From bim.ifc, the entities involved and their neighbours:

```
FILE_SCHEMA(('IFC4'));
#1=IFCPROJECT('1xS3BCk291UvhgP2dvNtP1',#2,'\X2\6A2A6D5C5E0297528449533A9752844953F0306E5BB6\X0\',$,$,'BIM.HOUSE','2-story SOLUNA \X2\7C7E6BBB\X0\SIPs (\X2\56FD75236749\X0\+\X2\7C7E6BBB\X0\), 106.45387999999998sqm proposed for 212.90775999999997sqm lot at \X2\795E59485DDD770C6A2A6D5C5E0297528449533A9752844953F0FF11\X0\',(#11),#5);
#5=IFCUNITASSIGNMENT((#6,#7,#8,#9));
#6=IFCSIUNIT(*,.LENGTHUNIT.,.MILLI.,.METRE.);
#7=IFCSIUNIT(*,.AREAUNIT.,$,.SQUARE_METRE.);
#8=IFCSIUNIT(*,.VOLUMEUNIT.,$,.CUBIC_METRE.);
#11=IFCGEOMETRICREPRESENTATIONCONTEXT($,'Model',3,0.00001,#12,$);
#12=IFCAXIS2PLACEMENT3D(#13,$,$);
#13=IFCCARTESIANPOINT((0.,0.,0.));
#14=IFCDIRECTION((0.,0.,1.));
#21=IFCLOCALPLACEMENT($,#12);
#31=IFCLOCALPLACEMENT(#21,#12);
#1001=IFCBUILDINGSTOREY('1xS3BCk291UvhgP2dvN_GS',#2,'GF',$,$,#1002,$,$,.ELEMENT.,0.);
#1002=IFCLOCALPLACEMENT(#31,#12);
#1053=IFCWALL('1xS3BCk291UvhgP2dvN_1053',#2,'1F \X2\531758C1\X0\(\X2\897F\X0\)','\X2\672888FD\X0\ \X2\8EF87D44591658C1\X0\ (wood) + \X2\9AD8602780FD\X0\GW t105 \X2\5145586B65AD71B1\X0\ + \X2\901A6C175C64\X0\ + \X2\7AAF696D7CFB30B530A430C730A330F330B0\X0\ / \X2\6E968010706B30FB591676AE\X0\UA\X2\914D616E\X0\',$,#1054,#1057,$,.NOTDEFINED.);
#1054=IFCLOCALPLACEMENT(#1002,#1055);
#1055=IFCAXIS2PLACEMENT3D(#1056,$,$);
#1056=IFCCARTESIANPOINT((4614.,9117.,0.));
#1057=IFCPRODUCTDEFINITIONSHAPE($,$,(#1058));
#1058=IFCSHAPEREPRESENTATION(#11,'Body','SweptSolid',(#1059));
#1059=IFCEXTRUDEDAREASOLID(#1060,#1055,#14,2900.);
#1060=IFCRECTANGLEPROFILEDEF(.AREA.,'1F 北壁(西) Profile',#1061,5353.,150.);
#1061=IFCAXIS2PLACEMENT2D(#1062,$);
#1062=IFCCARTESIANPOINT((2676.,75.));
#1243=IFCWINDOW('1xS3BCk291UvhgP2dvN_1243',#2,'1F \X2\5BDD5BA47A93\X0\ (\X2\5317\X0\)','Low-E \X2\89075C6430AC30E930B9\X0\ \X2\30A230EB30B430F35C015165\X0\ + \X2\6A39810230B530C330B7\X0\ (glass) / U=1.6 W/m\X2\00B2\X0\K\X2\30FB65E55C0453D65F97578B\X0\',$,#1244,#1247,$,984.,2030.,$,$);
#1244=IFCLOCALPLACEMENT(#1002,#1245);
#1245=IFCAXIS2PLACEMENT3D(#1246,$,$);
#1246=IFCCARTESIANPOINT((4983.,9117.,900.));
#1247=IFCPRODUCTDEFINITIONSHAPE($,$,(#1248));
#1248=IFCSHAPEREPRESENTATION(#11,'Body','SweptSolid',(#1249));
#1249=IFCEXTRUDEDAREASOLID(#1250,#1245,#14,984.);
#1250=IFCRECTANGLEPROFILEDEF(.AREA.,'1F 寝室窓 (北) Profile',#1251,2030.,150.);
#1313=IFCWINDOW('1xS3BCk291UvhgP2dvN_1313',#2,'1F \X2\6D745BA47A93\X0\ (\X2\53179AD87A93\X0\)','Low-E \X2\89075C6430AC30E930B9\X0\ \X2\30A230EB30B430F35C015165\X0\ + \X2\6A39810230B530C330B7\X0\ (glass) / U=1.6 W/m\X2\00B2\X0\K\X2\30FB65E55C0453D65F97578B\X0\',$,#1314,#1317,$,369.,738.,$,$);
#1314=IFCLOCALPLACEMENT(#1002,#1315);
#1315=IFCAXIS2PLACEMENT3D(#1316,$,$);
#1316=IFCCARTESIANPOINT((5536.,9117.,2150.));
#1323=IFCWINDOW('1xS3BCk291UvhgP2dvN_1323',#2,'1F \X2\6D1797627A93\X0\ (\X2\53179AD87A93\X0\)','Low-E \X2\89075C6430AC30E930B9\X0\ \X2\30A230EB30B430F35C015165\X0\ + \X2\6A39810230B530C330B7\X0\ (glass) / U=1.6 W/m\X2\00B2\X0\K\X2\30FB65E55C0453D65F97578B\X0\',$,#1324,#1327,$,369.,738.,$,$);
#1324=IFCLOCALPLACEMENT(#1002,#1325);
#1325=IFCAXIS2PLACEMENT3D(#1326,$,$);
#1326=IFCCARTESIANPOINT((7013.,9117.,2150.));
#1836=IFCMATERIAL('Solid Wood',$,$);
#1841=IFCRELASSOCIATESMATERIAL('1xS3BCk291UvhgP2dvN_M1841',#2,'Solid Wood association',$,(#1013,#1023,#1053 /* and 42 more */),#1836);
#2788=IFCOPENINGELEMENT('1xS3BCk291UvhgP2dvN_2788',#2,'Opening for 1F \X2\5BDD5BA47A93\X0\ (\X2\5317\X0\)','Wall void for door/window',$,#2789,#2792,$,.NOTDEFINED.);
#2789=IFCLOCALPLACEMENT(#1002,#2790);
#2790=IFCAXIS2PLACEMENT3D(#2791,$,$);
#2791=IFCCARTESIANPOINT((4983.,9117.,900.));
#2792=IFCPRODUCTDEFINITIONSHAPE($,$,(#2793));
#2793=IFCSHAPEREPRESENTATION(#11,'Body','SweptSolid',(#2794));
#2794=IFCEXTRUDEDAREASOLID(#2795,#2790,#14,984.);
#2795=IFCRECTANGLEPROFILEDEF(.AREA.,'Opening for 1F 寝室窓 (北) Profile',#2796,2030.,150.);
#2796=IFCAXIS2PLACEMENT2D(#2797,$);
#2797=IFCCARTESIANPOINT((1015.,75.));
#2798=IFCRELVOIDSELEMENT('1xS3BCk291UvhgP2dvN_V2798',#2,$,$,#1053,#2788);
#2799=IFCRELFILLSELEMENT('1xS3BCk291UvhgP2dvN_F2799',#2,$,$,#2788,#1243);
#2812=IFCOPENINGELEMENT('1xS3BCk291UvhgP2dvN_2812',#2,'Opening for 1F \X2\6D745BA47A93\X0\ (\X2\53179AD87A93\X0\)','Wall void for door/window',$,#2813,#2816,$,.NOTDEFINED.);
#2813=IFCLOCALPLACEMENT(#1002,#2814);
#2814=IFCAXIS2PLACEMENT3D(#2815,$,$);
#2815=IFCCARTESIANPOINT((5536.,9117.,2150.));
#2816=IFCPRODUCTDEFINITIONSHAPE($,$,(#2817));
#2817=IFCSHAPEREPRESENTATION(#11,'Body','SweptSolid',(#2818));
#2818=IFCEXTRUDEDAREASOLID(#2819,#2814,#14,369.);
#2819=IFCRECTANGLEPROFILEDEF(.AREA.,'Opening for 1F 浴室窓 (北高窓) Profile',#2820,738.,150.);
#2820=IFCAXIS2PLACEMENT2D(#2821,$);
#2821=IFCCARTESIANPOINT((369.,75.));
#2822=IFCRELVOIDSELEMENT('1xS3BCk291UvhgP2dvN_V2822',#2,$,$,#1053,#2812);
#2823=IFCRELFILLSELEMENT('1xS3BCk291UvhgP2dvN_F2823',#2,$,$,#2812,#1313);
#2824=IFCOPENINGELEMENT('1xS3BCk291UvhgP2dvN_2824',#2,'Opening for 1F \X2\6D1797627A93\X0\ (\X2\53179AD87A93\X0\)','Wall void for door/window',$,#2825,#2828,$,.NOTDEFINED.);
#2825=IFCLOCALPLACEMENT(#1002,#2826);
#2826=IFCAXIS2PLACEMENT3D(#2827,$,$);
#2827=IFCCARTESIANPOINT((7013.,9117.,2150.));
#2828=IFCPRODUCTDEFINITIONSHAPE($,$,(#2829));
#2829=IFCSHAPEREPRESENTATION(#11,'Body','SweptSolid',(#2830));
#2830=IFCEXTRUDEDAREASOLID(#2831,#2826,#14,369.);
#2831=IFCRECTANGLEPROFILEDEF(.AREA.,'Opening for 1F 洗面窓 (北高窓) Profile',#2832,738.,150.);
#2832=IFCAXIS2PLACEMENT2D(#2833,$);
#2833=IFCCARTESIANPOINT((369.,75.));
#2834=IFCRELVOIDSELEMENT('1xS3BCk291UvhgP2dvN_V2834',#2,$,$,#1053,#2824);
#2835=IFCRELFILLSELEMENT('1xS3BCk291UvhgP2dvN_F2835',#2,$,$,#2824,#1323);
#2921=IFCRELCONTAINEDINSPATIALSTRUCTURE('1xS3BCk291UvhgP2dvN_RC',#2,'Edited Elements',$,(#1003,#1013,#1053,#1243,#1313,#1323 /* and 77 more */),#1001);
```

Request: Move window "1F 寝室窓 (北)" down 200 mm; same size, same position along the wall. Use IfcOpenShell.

```python
import numpy as np
import ifcopenshell
import ifcopenshell.api.geometry
import ifcopenshell.util.placement
import ifcopenshell.util.unit

model = ifcopenshell.open("bim.ifc")
unit_scale = ifcopenshell.util.unit.calculate_unit_scale(model)

window = model.by_guid("1xS3BCk291UvhgP2dvN_1243")
opening = window.FillsVoids[0].RelatingOpeningElement
dz = -0.2 / unit_scale

shift = np.array([0.0, 0.0, dz])
# The window is not placed relative to its opening, so move both.
for product in (opening, window):
    matrix = ifcopenshell.util.placement.get_local_placement(product.ObjectPlacement)
    matrix[:3, 3] += shift
    ifcopenshell.api.geometry.edit_object_placement(model, product=product, matrix=matrix, is_si=False)

print(f"moved by {dz * unit_scale:+.3f} m")

model.write("bim_updated.ifc")
```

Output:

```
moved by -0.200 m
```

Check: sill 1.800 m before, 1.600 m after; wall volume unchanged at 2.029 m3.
